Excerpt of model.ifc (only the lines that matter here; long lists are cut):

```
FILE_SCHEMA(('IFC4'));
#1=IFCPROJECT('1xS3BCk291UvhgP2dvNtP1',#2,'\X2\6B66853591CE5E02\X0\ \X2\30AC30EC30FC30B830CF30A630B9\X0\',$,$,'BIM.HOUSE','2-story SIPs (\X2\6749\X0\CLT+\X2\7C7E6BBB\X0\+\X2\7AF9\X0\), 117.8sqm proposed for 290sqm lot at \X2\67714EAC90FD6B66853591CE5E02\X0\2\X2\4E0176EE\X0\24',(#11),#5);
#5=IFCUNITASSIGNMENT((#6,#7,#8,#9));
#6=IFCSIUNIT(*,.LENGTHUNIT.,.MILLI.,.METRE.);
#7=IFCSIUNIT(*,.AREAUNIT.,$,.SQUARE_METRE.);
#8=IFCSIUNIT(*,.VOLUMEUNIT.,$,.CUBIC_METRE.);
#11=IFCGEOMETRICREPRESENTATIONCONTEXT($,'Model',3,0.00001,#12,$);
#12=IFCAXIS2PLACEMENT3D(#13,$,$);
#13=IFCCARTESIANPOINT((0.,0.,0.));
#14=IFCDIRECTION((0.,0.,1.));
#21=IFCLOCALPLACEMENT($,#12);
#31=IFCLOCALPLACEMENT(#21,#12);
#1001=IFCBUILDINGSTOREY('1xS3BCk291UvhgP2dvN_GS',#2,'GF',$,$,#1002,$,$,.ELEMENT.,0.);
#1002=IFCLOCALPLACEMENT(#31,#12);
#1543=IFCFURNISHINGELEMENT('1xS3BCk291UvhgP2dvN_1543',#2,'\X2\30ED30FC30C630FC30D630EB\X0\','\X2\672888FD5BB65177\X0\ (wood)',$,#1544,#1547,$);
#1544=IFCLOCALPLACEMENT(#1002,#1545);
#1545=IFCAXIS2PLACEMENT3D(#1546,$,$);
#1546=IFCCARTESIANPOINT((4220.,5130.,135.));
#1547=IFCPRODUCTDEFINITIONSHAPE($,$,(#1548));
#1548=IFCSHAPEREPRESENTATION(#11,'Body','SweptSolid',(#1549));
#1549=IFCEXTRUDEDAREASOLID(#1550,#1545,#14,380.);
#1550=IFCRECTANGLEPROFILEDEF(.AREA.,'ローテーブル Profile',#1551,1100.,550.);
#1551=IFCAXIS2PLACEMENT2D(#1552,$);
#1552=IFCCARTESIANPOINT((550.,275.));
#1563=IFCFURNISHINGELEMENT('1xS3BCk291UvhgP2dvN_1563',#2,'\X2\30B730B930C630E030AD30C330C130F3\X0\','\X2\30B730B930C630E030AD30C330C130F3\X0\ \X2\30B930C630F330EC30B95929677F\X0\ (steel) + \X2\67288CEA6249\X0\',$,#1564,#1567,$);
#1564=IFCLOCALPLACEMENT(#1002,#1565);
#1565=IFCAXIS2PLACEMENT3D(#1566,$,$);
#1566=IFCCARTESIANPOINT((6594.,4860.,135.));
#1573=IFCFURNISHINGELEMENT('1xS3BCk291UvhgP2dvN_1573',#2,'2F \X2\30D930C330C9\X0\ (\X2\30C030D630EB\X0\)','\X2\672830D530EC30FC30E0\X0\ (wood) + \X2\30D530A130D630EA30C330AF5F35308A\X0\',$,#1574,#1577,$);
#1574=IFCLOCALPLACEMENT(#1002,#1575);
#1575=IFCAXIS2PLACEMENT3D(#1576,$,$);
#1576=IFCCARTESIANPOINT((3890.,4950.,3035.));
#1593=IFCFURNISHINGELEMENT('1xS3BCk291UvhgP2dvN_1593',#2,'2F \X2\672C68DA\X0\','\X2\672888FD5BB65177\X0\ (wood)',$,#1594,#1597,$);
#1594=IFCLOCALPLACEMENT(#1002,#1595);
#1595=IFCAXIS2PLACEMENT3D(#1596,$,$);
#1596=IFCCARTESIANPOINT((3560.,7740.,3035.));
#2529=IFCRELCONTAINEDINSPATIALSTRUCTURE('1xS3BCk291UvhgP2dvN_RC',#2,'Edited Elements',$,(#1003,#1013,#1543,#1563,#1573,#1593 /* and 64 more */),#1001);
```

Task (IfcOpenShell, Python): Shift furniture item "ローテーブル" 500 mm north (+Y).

```python
import ifcopenshell
import ifcopenshell.api.geometry
import ifcopenshell.util.placement
import ifcopenshell.util.unit

model = ifcopenshell.open("model.ifc")
unit_scale = ifcopenshell.util.unit.calculate_unit_scale(model)

item = model.by_guid("1xS3BCk291UvhgP2dvN_1543")
matrix = ifcopenshell.util.placement.get_local_placement(item.ObjectPlacement)
matrix[1, 3] += 0.5 / unit_scale
ifcopenshell.api.geometry.edit_object_placement(model, product=item, matrix=matrix, is_si=False)

print(ifcopenshell.util.placement.get_local_placement(item.ObjectPlacement).round(3) + 0.0)

model.write("model-out.ifc")
```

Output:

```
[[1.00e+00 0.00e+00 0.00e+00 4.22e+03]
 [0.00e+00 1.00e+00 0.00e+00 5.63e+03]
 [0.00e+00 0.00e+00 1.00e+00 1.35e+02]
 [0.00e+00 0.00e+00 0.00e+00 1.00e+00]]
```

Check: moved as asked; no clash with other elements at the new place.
